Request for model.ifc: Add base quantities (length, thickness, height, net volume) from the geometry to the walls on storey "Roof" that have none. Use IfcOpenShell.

First a look at what the model holds.

```python
import ifcopenshell
import ifcopenshell.util.element
import ifcopenshell.util.unit

model = ifcopenshell.open("model.ifc")
print(model.schema)
for unit_type in ("LENGTHUNIT", "AREAUNIT", "VOLUMEUNIT"):
    print(unit_type, ifcopenshell.util.unit.calculate_unit_scale(model, unit_type))
storey = next(s for s in model.by_type("IfcBuildingStorey") if s.Name == "Roof")
walls = [e for e in ifcopenshell.util.element.get_decomposition(storey) if e.is_a("IfcWall")]
for e in sorted(walls, key=lambda e: e.id()):
    print(e.id(), e.is_a(), e.Name, list(ifcopenshell.util.element.get_psets(e, qtos_only=True)), sep=" | ")
```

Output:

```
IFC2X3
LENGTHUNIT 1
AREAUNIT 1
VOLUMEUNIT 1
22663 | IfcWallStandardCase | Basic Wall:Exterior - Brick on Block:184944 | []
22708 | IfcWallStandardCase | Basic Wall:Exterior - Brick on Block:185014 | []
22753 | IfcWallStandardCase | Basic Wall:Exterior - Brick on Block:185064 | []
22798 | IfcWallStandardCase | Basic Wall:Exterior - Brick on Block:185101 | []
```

```python
import ifcopenshell
import ifcopenshell.api.pset
import ifcopenshell.geom
import ifcopenshell.util.element
import ifcopenshell.util.shape
import ifcopenshell.util.unit

model = ifcopenshell.open("model.ifc")
unit_scale = ifcopenshell.util.unit.calculate_unit_scale(model)
volume_scale = ifcopenshell.util.unit.calculate_unit_scale(model, "VOLUMEUNIT")
settings = ifcopenshell.geom.settings()

storey = next(s for s in model.by_type("IfcBuildingStorey") if s.Name == "Roof")
walls = [e for e in ifcopenshell.util.element.get_decomposition(storey) if e.is_a("IfcWall")]

for e in sorted(walls, key=lambda e: e.id()):
    if ifcopenshell.util.element.get_psets(e, qtos_only=True, should_inherit=False):
        continue
    # Geometry comes back in metres, in the element's own axes.
    shape = ifcopenshell.geom.create_shape(settings, e)
    values = {
        "Length": ifcopenshell.util.shape.get_x(shape.geometry) / unit_scale,
        "Width": ifcopenshell.util.shape.get_y(shape.geometry) / unit_scale,
        "Height": ifcopenshell.util.shape.get_z(shape.geometry) / unit_scale,
        "NetVolume": ifcopenshell.util.shape.get_volume(shape.geometry) / volume_scale,
    }
    qto = ifcopenshell.api.pset.add_qto(model, product=e, name="BaseQuantities")
    ifcopenshell.api.pset.edit_qto(model, qto=qto, properties=values)
    print(e.id(), {k: round(v, 3) for k, v in values.items()})

model.write("model_updated.ifc")
```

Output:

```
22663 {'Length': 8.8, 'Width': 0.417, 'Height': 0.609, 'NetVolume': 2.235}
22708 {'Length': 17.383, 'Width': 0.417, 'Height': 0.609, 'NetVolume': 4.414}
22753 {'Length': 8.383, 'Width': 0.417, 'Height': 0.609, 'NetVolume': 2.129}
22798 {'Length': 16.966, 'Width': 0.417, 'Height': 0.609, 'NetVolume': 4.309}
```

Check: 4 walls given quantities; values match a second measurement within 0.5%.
